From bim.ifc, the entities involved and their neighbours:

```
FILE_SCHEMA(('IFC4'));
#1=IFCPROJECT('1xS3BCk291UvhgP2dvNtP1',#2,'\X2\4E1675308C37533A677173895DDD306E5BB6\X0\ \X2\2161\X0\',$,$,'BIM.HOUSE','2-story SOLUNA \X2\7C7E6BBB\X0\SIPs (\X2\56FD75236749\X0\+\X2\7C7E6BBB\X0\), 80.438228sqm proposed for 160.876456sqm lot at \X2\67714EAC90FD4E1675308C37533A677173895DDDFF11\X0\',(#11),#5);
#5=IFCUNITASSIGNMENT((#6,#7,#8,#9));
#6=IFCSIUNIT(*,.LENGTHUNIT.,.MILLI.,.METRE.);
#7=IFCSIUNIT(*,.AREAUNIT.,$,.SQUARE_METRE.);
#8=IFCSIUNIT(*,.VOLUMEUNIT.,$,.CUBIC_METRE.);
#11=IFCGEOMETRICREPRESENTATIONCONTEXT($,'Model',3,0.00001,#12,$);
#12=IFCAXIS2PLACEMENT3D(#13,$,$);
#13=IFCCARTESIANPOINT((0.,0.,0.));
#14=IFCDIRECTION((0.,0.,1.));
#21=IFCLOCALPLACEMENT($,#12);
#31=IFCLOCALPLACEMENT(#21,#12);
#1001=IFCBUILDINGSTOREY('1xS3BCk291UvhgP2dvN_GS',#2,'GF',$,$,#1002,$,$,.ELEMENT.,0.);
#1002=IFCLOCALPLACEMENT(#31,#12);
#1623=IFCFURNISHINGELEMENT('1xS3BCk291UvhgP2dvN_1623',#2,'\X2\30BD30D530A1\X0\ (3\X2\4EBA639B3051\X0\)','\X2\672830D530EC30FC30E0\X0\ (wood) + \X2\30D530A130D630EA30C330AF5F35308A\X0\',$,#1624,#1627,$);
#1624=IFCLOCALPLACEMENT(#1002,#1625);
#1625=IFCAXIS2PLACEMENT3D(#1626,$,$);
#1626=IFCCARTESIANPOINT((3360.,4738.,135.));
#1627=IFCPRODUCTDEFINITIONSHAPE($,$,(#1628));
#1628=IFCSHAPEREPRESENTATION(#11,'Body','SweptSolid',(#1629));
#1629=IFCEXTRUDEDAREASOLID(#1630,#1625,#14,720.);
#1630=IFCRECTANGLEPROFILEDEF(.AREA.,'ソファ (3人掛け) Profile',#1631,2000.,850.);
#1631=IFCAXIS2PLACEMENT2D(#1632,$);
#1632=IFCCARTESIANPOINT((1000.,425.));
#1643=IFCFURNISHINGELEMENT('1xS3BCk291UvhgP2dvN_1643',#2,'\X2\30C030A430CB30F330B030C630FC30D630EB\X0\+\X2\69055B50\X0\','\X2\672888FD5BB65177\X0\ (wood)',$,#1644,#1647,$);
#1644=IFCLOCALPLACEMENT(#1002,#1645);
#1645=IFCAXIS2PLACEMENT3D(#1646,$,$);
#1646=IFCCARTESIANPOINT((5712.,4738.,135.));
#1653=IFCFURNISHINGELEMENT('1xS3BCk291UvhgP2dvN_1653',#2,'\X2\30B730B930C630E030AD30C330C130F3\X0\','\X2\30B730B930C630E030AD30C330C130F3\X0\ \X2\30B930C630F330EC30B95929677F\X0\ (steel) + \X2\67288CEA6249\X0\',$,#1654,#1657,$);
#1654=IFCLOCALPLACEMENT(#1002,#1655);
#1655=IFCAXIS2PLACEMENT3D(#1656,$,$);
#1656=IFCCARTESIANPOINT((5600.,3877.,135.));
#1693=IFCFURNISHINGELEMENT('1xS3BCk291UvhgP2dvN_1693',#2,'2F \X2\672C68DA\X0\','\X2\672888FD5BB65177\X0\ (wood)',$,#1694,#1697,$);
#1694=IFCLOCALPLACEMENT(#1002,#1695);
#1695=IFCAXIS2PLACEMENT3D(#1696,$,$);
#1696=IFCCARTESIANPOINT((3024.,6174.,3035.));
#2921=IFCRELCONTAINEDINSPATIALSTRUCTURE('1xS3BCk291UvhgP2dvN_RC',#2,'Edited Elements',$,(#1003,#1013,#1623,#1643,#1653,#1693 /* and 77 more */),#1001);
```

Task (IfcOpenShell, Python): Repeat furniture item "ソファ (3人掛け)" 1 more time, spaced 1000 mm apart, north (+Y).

```python
import numpy as np
import ifcopenshell
import ifcopenshell.api.geometry
import ifcopenshell.api.root
import ifcopenshell.util.element
import ifcopenshell.util.placement

model = ifcopenshell.open("bim.ifc")


def reuse_history(source, copy):
    """copy_class also copies each property set's owner history, people and application; keep the originals."""
    for rel in copy.IsDefinedBy:
        if rel.is_a("IfcRelDefinesByProperties") and (history := rel.RelatingPropertyDefinition.OwnerHistory):
            rel.RelatingPropertyDefinition.OwnerHistory = source.OwnerHistory
            ifcopenshell.util.element.remove_deep2(model, history)


source = model.by_guid("1xS3BCk291UvhgP2dvN_1623")
base = ifcopenshell.util.placement.get_local_placement(source.ObjectPlacement)
step = np.array([0.0, 1.0, 0.0]) * 1000.0

for i in range(1, 2):
    copy = ifcopenshell.api.root.copy_class(model, product=source)
    copy.Representation = ifcopenshell.util.element.copy_deep(
        model, source.Representation, exclude=["IfcGeometricRepresentationContext", "IfcRepresentationMap"]
    )
    reuse_history(source, copy)
    matrix = base.copy()
    matrix[:3, 3] += i * step
    print("added at", matrix[:3, 3].round(3) + 0.0)
    ifcopenshell.api.geometry.edit_object_placement(model, product=copy, matrix=matrix, is_si=False)

model.write("bim_updated.ifc")
```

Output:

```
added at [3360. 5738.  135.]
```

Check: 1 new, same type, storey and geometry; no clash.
